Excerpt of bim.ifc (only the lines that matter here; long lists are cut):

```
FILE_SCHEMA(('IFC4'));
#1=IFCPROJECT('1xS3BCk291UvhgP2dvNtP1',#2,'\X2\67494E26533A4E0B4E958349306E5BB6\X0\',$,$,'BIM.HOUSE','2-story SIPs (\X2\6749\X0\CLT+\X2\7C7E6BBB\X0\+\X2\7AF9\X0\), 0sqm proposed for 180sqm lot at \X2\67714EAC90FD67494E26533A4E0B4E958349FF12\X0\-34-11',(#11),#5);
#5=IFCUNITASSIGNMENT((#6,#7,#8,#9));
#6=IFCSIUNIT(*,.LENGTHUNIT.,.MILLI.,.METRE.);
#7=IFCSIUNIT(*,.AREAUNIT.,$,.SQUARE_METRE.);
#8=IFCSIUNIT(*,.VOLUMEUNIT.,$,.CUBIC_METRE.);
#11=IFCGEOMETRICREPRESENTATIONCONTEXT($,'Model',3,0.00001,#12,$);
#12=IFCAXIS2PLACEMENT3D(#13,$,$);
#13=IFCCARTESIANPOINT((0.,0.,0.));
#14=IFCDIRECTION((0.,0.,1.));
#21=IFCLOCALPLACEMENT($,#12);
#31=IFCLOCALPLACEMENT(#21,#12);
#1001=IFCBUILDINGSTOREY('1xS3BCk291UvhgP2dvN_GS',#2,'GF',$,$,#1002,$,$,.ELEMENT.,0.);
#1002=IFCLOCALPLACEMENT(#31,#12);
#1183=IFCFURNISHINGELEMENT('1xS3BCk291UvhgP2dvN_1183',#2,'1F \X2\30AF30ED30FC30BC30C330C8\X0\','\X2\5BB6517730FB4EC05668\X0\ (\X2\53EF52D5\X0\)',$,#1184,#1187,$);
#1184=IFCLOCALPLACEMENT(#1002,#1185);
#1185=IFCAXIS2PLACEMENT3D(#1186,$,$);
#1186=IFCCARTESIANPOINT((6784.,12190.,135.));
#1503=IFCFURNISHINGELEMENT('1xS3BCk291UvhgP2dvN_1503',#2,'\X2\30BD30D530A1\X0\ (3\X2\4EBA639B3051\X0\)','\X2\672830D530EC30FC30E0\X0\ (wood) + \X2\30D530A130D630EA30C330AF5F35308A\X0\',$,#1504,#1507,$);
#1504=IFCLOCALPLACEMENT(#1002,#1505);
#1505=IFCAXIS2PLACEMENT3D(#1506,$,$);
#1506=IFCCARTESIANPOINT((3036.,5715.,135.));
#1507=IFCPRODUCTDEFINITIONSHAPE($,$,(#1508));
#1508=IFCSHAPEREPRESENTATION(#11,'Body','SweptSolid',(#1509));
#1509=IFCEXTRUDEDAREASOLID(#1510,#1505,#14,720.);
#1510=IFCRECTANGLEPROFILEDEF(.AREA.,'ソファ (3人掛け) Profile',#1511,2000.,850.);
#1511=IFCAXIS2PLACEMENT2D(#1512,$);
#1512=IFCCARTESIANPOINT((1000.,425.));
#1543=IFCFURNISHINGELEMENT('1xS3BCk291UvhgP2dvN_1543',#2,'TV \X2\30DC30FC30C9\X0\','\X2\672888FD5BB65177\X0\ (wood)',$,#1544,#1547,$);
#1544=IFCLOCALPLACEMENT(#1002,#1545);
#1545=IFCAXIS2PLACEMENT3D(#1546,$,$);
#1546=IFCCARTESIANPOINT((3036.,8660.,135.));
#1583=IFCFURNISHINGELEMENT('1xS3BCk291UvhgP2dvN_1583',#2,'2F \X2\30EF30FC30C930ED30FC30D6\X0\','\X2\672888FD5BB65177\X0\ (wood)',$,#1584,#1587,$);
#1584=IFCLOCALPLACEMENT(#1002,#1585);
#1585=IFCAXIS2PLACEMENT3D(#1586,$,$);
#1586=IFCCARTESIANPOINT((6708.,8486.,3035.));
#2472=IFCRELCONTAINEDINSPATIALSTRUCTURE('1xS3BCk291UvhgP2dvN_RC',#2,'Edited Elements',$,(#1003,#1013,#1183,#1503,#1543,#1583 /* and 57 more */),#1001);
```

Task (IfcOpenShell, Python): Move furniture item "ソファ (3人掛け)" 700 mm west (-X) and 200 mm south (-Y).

```python
import ifcopenshell
import ifcopenshell.api.geometry
import ifcopenshell.util.placement
import ifcopenshell.util.unit

model = ifcopenshell.open("bim.ifc")
unit_scale = ifcopenshell.util.unit.calculate_unit_scale(model)

item = model.by_id(1503)
matrix = ifcopenshell.util.placement.get_local_placement(item.ObjectPlacement)
matrix[0, 3] -= 0.7 / unit_scale
matrix[1, 3] -= 0.2 / unit_scale
ifcopenshell.api.geometry.edit_object_placement(model, product=item, matrix=matrix, is_si=False)

print(ifcopenshell.util.placement.get_local_placement(item.ObjectPlacement).round(3) + 0.0)

model.write("bim_rev.ifc")
```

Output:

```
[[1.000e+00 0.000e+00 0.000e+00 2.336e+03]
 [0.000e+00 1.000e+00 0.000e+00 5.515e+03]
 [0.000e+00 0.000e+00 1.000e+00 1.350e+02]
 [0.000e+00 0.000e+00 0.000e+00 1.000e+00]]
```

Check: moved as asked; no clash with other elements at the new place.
